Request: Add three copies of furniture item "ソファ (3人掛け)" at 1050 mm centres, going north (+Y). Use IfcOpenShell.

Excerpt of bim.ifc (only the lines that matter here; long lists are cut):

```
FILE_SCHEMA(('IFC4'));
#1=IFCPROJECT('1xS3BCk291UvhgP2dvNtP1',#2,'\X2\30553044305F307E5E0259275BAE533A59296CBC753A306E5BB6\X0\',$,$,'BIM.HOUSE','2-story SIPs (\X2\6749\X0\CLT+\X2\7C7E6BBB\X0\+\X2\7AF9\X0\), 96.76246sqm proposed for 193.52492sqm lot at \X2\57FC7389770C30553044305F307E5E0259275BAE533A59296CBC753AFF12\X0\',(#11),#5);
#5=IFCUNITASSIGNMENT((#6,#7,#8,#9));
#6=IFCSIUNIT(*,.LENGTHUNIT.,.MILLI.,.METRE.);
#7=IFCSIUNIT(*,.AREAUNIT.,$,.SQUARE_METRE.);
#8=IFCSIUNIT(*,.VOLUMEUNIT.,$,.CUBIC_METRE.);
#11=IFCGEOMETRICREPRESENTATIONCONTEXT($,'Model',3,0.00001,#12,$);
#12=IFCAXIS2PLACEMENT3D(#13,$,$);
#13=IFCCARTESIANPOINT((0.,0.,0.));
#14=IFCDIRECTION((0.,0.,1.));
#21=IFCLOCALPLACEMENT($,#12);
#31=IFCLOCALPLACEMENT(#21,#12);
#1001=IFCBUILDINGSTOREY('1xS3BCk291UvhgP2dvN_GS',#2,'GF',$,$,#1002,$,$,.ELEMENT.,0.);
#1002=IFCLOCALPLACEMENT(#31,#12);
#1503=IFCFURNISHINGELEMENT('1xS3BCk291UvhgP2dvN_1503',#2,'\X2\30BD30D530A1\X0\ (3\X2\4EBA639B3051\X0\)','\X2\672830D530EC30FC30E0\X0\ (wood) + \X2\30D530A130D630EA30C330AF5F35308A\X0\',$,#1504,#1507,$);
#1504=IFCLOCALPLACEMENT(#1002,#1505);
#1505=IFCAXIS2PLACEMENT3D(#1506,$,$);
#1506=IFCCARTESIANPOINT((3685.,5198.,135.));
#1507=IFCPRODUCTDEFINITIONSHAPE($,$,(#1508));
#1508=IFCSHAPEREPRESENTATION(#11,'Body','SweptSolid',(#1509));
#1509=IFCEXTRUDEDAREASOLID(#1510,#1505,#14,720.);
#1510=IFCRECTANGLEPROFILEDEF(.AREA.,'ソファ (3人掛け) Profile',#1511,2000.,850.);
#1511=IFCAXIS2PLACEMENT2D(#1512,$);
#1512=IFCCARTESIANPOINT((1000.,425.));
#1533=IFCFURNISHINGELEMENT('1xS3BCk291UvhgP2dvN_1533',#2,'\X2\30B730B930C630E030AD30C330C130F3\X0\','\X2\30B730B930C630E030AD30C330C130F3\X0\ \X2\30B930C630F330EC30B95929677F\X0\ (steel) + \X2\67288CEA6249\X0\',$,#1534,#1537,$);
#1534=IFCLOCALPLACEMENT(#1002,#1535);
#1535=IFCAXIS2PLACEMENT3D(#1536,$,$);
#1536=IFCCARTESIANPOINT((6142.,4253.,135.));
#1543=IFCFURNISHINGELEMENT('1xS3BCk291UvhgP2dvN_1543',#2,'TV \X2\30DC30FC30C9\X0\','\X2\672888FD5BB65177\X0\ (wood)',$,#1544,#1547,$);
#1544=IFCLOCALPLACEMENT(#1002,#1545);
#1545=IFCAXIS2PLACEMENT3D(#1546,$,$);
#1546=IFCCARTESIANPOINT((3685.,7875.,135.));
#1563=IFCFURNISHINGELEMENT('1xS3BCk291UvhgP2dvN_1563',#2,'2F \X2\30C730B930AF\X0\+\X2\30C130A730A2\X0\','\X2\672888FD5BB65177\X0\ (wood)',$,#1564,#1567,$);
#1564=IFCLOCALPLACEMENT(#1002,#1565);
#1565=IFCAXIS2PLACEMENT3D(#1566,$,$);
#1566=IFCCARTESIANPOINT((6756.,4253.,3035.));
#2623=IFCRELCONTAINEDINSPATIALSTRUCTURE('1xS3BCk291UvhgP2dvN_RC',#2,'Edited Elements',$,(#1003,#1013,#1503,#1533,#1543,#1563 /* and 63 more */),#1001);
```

```python
import numpy as np
import ifcopenshell
import ifcopenshell.api.geometry
import ifcopenshell.api.root
import ifcopenshell.util.element
import ifcopenshell.util.placement
import ifcopenshell.util.unit

model = ifcopenshell.open("bim.ifc")
unit_scale = ifcopenshell.util.unit.calculate_unit_scale(model)


def reuse_history(source, copy):
    """copy_class also copies each property set's owner history, people and application; keep the originals."""
    for rel in copy.IsDefinedBy:
        if rel.is_a("IfcRelDefinesByProperties") and (history := rel.RelatingPropertyDefinition.OwnerHistory):
            rel.RelatingPropertyDefinition.OwnerHistory = source.OwnerHistory
            ifcopenshell.util.element.remove_deep2(model, history)


source = model.by_id(1503)
base = ifcopenshell.util.placement.get_local_placement(source.ObjectPlacement)
step = np.array([0.0, 1.0, 0.0]) * 1.05 / unit_scale

for i in range(1, 4):
    copy = ifcopenshell.api.root.copy_class(model, product=source)
    copy.Representation = ifcopenshell.util.element.copy_deep(
        model, source.Representation, exclude=["IfcGeometricRepresentationContext", "IfcRepresentationMap"]
    )
    reuse_history(source, copy)
    matrix = base.copy()
    matrix[:3, 3] += i * step
    print("added at", matrix[:3, 3].round(3) + 0.0)
    ifcopenshell.api.geometry.edit_object_placement(model, product=copy, matrix=matrix, is_si=False)

model.write("bim_edited.ifc")
```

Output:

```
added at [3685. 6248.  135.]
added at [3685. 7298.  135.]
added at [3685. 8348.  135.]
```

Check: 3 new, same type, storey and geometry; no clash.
